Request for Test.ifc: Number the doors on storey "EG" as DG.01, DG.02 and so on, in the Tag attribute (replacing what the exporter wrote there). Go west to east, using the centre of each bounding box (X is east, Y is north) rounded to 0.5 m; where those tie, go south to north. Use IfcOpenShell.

First a look at what the model holds.

```python
import ifcopenshell
import ifcopenshell.util.element
import ifcopenshell.util.placement

model = ifcopenshell.open("Test.ifc")
print(model.schema)
storey = next(s for s in model.by_type("IfcBuildingStorey") if s.Name == "EG")
doors = [e for e in ifcopenshell.util.element.get_decomposition(storey) if e.is_a("IfcDoor")]
for e in sorted(doors, key=lambda e: e.id()):
    origin = ifcopenshell.util.placement.get_local_placement(e.ObjectPlacement)[:3, 3]
    print(e.id(), e.Tag, e.Name, origin.round(2) + 0.0, sep=" | ")
```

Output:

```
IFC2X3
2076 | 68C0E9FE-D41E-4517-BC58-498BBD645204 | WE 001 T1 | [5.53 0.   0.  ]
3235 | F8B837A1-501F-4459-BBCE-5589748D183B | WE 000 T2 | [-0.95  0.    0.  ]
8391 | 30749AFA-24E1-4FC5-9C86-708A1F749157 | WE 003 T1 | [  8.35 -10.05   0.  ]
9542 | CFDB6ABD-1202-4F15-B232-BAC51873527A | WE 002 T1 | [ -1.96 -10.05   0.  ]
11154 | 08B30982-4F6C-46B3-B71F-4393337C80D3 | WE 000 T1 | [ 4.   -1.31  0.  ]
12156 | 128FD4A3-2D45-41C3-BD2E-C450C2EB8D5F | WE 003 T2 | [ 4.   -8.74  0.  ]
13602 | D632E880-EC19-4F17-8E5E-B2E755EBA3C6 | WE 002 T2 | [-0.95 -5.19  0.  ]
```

```python
import ifcopenshell
import ifcopenshell.geom
import ifcopenshell.util.element
import ifcopenshell.util.shape

model = ifcopenshell.open("Test.ifc")
settings = ifcopenshell.geom.settings()
settings.set("use-world-coords", True)


def centre(element):
    shape = ifcopenshell.geom.create_shape(settings, element)
    return ifcopenshell.util.shape.get_bbox_centroid(shape.geometry)


storey = next(s for s in model.by_type("IfcBuildingStorey") if s.Name == "EG")
doors = [e for e in ifcopenshell.util.element.get_decomposition(storey) if e.is_a("IfcDoor")]

# Insertion points can sit at a corner or the storey origin, so sort by the geometry (in metres).
centres = {e: centre(e) for e in doors}
doors.sort(key=lambda e: (round(centres[e][0] / 0.5), centres[e][1]))

for i, e in enumerate(doors, start=1):
    number = f"DG.{i:02d}"
    e.Tag = number
    print(e.id(), number)

model.write("Test_rev.ifc")
```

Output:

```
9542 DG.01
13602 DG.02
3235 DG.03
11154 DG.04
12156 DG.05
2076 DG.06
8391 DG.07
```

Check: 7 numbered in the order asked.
